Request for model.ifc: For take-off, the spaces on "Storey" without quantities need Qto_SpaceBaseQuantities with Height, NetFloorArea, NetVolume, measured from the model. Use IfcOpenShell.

First a look at what the model holds.

```python
import ifcopenshell
import ifcopenshell.util.element
import ifcopenshell.util.unit

model = ifcopenshell.open("model.ifc")
print(model.schema)
for unit_type in ("LENGTHUNIT", "AREAUNIT", "VOLUMEUNIT"):
    print(unit_type, ifcopenshell.util.unit.calculate_unit_scale(model, unit_type))
storey = next(s for s in model.by_type("IfcBuildingStorey") if s.Name == "Storey")
spaces = [e for e in ifcopenshell.util.element.get_decomposition(storey) if e.is_a("IfcSpace")]
for e in sorted(spaces, key=lambda e: e.id()):
    print(e.id(), e.is_a(), e.Name, list(ifcopenshell.util.element.get_psets(e, qtos_only=True)), sep=" | ")
```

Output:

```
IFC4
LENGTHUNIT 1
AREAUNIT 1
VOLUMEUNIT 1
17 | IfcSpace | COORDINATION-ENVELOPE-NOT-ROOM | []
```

```python
import ifcopenshell
import ifcopenshell.api.pset
import ifcopenshell.geom
import ifcopenshell.util.element
import ifcopenshell.util.shape
import ifcopenshell.util.unit

model = ifcopenshell.open("model.ifc")
unit_scale = ifcopenshell.util.unit.calculate_unit_scale(model)
area_scale = ifcopenshell.util.unit.calculate_unit_scale(model, "AREAUNIT")
volume_scale = ifcopenshell.util.unit.calculate_unit_scale(model, "VOLUMEUNIT")
settings = ifcopenshell.geom.settings()

storey = next(s for s in model.by_type("IfcBuildingStorey") if s.Name == "Storey")
spaces = [e for e in ifcopenshell.util.element.get_decomposition(storey) if e.is_a("IfcSpace")]

for e in sorted(spaces, key=lambda e: e.id()):
    if ifcopenshell.util.element.get_psets(e, qtos_only=True, should_inherit=False):
        continue
    # Geometry comes back in metres, in the element's own axes.
    shape = ifcopenshell.geom.create_shape(settings, e)
    values = {
        "Height": ifcopenshell.util.shape.get_z(shape.geometry) / unit_scale,
        "NetFloorArea": ifcopenshell.util.shape.get_footprint_area(shape.geometry) / area_scale,
        "NetVolume": ifcopenshell.util.shape.get_volume(shape.geometry) / volume_scale,
    }
    qto = ifcopenshell.api.pset.add_qto(model, product=e, name="Qto_SpaceBaseQuantities")
    ifcopenshell.api.pset.edit_qto(model, qto=qto, properties=values)
    print(e.id(), {k: round(v, 3) for k, v in values.items()})

model.write("model_rev.ifc")
```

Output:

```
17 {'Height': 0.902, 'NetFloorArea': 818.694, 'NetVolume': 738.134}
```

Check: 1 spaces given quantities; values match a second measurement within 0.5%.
